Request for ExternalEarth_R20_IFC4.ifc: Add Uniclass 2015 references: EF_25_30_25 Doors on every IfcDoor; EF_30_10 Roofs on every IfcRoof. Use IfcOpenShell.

First a look at what the model holds.

```python
import ifcopenshell

model = ifcopenshell.open("ExternalEarth_R20_IFC4.ifc")
print(model.schema)
print("classifications:", [c.Name for c in model.by_type("IfcClassification")])
for ifc_class in ("IfcDoor", "IfcRoof", "IfcStair", "IfcWall", "IfcWindow"):
    print(ifc_class, len(model.by_type(ifc_class)))
```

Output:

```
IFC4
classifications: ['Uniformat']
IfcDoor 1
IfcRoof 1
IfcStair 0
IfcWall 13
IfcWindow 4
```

```python
import ifcopenshell
import ifcopenshell.api.classification

model = ifcopenshell.open("ExternalEarth_R20_IFC4.ifc")

system = ifcopenshell.api.classification.add_classification(model, classification="Uniclass 2015")

codes = {
    "IfcDoor": ("EF_25_30_25", "Doors"),
    "IfcRoof": ("EF_30_10", "Roofs"),
}
for ifc_class, (code, name) in codes.items():
    products = model.by_type(ifc_class)
    ifcopenshell.api.classification.add_reference(
        model, products=products, classification=system, identification=code, name=name
    )
    print(code, len(products))

model.write("ExternalEarth_R20_IFC4-out.ifc")
```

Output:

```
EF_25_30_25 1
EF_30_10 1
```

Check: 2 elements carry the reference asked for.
